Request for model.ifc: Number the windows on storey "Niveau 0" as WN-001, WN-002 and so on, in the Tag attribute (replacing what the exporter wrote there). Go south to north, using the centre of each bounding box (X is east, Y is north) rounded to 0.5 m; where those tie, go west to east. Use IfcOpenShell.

First a look at what the model holds.

```python
import ifcopenshell
import ifcopenshell.util.element
import ifcopenshell.util.placement

model = ifcopenshell.open("model.ifc")
print(model.schema)
storey = next(s for s in model.by_type("IfcBuildingStorey") if s.Name == "Niveau 0")
windows = [e for e in ifcopenshell.util.element.get_decomposition(storey) if e.is_a("IfcWindow")]
for e in sorted(windows, key=lambda e: e.id()):
    origin = ifcopenshell.util.placement.get_local_placement(e.ObjectPlacement)[:3, 3]
    print(e.id(), e.Tag, e.Name, origin.round(2) + 0.0, sep=" | ")
```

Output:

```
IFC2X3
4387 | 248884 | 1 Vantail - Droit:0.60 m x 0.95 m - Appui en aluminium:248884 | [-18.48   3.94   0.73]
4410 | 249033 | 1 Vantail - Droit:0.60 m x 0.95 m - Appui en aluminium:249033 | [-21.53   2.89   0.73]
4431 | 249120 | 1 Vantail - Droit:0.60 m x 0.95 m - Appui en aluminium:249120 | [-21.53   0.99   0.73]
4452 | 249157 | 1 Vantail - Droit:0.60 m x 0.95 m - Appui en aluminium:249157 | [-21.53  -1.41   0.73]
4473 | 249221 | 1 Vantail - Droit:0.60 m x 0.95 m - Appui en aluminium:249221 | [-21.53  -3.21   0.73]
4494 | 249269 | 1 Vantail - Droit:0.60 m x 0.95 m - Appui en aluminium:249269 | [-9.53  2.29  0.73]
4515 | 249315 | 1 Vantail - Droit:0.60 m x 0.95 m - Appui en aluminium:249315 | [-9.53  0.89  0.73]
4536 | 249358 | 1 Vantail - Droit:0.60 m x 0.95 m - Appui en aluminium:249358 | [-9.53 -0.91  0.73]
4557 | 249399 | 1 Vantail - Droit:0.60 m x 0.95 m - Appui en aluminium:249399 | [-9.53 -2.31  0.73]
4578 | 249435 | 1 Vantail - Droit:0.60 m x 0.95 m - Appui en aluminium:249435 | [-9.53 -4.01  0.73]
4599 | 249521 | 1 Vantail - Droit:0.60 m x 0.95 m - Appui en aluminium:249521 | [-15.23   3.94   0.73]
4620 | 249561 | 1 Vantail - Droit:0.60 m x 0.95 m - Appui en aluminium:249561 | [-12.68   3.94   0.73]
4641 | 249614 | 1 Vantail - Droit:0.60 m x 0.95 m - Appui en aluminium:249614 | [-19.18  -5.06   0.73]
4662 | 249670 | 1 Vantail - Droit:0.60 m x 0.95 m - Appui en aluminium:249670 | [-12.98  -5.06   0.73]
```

```python
import ifcopenshell
import ifcopenshell.geom
import ifcopenshell.util.element
import ifcopenshell.util.shape

model = ifcopenshell.open("model.ifc")
settings = ifcopenshell.geom.settings()
settings.set("use-world-coords", True)


def centre(element):
    shape = ifcopenshell.geom.create_shape(settings, element)
    return ifcopenshell.util.shape.get_bbox_centroid(shape.geometry)


storey = next(s for s in model.by_type("IfcBuildingStorey") if s.Name == "Niveau 0")
windows = [e for e in ifcopenshell.util.element.get_decomposition(storey) if e.is_a("IfcWindow")]

# Insertion points can sit at a corner or the storey origin, so sort by the geometry (in metres).
centres = {e: centre(e) for e in windows}
windows.sort(key=lambda e: (round(centres[e][1] / 0.5), centres[e][0]))

for i, e in enumerate(windows, start=1):
    number = f"WN-0{i:02d}"
    e.Tag = number
    print(e.id(), number)

model.write("model-out.ifc")
```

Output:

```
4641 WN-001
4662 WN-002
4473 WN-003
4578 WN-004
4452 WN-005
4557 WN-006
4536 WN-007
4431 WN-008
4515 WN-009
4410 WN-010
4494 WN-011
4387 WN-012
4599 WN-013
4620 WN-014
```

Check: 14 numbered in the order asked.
